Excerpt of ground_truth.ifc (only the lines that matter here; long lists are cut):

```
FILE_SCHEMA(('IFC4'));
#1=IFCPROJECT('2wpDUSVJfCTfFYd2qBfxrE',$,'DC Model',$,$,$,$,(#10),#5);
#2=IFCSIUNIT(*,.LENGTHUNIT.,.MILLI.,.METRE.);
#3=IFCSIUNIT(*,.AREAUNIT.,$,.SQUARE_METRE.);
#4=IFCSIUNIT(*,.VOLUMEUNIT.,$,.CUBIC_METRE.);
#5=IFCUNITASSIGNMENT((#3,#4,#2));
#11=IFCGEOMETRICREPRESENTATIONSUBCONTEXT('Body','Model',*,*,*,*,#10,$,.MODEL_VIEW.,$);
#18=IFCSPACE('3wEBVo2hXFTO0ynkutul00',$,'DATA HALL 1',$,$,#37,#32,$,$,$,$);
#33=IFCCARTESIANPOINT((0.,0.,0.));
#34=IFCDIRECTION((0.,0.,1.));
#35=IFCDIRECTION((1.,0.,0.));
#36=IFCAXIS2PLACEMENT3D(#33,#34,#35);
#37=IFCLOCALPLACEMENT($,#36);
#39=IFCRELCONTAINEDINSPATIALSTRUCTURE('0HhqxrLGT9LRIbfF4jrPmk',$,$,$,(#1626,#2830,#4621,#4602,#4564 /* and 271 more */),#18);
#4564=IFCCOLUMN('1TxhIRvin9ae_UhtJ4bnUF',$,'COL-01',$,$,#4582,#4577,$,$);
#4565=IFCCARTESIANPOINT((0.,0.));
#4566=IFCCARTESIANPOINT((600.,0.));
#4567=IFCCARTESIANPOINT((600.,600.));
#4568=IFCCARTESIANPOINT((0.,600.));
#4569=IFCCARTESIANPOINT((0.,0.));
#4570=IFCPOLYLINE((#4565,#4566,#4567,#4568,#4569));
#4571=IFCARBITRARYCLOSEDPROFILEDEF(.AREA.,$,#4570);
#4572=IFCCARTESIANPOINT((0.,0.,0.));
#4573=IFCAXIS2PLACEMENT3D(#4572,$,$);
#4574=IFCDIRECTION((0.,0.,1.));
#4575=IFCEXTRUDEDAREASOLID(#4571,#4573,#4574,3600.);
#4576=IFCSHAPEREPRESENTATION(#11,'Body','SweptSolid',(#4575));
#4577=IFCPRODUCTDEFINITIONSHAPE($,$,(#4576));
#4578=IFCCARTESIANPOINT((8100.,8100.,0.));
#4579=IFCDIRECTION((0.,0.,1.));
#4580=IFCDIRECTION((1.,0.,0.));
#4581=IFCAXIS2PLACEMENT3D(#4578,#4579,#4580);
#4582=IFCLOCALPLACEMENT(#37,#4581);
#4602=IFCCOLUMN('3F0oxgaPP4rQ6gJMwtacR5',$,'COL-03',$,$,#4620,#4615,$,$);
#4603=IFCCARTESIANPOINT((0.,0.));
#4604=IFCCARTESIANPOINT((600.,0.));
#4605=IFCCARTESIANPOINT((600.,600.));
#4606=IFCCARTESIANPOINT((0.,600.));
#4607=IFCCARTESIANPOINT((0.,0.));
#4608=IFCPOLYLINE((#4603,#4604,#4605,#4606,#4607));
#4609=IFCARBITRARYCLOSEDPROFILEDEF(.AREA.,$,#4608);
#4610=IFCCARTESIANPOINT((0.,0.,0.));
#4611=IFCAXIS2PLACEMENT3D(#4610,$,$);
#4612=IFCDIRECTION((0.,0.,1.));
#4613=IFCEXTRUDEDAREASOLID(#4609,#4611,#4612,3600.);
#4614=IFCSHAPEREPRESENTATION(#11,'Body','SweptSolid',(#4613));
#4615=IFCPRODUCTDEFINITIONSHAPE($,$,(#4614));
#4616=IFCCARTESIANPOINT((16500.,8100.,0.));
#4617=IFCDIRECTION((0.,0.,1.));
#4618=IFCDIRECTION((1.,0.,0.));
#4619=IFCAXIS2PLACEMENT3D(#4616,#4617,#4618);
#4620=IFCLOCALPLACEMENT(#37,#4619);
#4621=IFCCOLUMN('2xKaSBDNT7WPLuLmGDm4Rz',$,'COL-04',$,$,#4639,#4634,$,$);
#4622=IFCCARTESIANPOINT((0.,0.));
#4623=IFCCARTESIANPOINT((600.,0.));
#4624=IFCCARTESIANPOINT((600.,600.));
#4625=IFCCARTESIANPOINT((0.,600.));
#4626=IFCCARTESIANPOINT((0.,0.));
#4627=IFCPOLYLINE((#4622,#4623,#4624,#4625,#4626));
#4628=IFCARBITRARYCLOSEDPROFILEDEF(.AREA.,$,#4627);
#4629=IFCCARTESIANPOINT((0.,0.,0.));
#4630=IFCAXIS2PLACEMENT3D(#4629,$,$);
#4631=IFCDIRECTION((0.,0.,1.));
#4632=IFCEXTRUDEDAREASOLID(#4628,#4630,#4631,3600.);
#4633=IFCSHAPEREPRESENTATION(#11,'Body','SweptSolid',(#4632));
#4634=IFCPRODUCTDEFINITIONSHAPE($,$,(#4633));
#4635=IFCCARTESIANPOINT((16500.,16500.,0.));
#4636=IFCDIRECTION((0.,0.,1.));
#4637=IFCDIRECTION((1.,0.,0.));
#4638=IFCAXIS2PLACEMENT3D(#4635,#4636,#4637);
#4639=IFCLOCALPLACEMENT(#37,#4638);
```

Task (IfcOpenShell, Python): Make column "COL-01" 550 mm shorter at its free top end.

```python
import ifcopenshell
import ifcopenshell.util.representation
import ifcopenshell.util.unit

model = ifcopenshell.open("ground_truth.ifc")
unit_scale = ifcopenshell.util.unit.calculate_unit_scale(model)

member = model.by_guid("1TxhIRvin9ae_UhtJ4bnUF")
change = -0.55 / unit_scale

# The extrusion runs towards the end named, so only its depth changes.
body = ifcopenshell.util.representation.get_representation(member, "Model", "Body")
solid = body.Items[0]
old_length = solid.Depth
solid.Depth += change

print(f"length {old_length:g} -> {solid.Depth:g}")

model.write("ground_truth-out.ifc")
```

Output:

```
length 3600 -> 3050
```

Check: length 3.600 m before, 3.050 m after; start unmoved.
